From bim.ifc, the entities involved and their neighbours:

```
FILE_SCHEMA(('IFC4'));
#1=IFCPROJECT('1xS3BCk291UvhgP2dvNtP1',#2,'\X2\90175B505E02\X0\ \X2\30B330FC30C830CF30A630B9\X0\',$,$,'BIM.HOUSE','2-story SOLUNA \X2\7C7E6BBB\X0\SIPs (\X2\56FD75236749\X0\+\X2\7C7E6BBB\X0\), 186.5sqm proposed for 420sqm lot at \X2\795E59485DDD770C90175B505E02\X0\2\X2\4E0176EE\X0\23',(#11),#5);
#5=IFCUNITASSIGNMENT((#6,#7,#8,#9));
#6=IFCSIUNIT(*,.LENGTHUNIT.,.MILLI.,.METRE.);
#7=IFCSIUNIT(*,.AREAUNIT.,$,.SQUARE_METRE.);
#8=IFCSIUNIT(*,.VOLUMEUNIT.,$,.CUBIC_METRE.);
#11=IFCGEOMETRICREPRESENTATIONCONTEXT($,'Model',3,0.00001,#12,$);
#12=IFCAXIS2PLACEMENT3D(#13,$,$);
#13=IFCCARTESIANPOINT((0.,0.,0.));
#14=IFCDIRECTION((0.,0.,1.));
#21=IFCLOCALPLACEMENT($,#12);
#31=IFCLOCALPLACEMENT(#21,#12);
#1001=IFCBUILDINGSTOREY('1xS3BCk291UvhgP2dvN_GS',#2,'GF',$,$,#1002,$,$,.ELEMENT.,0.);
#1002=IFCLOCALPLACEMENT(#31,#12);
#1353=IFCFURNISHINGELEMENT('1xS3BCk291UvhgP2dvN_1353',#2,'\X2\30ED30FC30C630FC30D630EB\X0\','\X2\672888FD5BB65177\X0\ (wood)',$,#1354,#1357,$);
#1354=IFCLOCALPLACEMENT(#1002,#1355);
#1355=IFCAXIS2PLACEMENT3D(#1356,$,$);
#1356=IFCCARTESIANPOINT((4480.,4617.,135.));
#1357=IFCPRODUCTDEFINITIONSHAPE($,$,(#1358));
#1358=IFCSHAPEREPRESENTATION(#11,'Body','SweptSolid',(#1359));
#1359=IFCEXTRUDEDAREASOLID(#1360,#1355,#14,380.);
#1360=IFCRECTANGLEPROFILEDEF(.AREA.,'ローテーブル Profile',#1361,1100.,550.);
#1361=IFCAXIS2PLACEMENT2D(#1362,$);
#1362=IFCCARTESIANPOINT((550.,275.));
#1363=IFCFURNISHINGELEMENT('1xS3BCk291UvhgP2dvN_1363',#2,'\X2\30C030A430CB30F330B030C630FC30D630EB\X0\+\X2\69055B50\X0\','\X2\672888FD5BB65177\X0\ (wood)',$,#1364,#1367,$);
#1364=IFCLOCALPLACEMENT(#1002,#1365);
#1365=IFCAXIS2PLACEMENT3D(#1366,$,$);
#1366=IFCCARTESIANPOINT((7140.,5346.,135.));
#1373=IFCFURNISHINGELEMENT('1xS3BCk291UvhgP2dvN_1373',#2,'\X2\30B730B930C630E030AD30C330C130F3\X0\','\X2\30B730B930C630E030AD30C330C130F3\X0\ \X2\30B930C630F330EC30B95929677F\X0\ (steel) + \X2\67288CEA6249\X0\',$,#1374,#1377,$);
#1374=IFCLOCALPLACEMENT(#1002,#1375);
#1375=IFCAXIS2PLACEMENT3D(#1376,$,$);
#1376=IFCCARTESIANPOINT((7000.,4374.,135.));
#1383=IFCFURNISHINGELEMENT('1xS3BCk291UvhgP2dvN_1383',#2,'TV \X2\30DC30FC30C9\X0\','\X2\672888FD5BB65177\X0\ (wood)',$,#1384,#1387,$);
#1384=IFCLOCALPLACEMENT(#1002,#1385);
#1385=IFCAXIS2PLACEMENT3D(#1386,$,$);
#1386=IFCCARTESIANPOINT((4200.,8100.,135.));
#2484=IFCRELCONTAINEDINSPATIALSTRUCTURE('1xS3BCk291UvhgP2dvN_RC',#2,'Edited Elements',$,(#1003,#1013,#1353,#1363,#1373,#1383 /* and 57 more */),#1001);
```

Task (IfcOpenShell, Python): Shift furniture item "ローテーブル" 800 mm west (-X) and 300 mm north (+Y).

```python
import ifcopenshell
import ifcopenshell.api.geometry
import ifcopenshell.util.placement

model = ifcopenshell.open("bim.ifc")

item = model.by_guid("1xS3BCk291UvhgP2dvN_1353")
matrix = ifcopenshell.util.placement.get_local_placement(item.ObjectPlacement)
matrix[0, 3] -= 800.0
matrix[1, 3] += 300.0
ifcopenshell.api.geometry.edit_object_placement(model, product=item, matrix=matrix, is_si=False)

print(ifcopenshell.util.placement.get_local_placement(item.ObjectPlacement).round(3) + 0.0)

model.write("bim_edited.ifc")
```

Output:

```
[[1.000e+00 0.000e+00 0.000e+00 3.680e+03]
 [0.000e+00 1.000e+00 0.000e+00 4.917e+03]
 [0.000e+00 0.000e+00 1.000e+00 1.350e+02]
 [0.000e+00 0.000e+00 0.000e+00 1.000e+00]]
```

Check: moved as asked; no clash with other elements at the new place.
